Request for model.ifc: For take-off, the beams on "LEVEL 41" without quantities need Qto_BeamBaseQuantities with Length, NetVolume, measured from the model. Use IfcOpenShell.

First a look at what the model holds.

```python
import ifcopenshell
import ifcopenshell.util.element
import ifcopenshell.util.unit

model = ifcopenshell.open("model.ifc")
print(model.schema)
for unit_type in ("LENGTHUNIT", "AREAUNIT", "VOLUMEUNIT"):
    print(unit_type, ifcopenshell.util.unit.calculate_unit_scale(model, unit_type))
storey = next(s for s in model.by_type("IfcBuildingStorey") if s.Name == "LEVEL 41")
beams = [e for e in ifcopenshell.util.element.get_decomposition(storey) if e.is_a("IfcBeam")]
for e in sorted(beams, key=lambda e: e.id()):
    print(e.id(), e.is_a(), e.Name, list(ifcopenshell.util.element.get_psets(e, qtos_only=True)), sep=" | ")
```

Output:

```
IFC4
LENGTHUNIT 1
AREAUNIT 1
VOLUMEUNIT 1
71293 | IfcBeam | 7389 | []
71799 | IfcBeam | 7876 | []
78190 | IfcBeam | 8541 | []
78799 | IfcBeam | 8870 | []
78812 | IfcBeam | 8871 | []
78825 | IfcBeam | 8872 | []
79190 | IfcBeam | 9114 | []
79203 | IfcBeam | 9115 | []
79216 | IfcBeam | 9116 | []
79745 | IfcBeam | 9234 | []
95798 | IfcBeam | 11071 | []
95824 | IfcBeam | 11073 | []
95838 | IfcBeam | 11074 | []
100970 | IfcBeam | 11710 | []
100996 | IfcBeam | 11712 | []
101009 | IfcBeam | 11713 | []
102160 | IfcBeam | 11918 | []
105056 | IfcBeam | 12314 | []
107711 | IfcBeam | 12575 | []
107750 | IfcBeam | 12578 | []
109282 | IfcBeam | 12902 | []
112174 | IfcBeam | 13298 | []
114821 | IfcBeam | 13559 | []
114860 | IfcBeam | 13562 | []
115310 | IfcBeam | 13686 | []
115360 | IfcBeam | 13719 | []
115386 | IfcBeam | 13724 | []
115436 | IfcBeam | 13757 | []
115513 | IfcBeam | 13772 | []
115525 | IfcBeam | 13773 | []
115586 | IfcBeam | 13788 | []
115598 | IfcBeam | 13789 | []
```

```python
import ifcopenshell
import ifcopenshell.api.pset
import ifcopenshell.geom
import ifcopenshell.util.element
import ifcopenshell.util.shape
import ifcopenshell.util.unit

model = ifcopenshell.open("model.ifc")
unit_scale = ifcopenshell.util.unit.calculate_unit_scale(model)
volume_scale = ifcopenshell.util.unit.calculate_unit_scale(model, "VOLUMEUNIT")
settings = ifcopenshell.geom.settings()

storey = next(s for s in model.by_type("IfcBuildingStorey") if s.Name == "LEVEL 41")
beams = [e for e in ifcopenshell.util.element.get_decomposition(storey) if e.is_a("IfcBeam")]

for e in sorted(beams, key=lambda e: e.id()):
    if ifcopenshell.util.element.get_psets(e, qtos_only=True, should_inherit=False):
        continue
    # Geometry comes back in metres, in the element's own axes.
    shape = ifcopenshell.geom.create_shape(settings, e)
    values = {
        "Length": ifcopenshell.util.shape.get_max_xyz(shape.geometry) / unit_scale,
        "NetVolume": ifcopenshell.util.shape.get_volume(shape.geometry) / volume_scale,
    }
    qto = ifcopenshell.api.pset.add_qto(model, product=e, name="Qto_BeamBaseQuantities")
    ifcopenshell.api.pset.edit_qto(model, qto=qto, properties=values)
    print(e.id(), {k: round(v, 3) for k, v in values.items()})

model.write("model-out.ifc")
```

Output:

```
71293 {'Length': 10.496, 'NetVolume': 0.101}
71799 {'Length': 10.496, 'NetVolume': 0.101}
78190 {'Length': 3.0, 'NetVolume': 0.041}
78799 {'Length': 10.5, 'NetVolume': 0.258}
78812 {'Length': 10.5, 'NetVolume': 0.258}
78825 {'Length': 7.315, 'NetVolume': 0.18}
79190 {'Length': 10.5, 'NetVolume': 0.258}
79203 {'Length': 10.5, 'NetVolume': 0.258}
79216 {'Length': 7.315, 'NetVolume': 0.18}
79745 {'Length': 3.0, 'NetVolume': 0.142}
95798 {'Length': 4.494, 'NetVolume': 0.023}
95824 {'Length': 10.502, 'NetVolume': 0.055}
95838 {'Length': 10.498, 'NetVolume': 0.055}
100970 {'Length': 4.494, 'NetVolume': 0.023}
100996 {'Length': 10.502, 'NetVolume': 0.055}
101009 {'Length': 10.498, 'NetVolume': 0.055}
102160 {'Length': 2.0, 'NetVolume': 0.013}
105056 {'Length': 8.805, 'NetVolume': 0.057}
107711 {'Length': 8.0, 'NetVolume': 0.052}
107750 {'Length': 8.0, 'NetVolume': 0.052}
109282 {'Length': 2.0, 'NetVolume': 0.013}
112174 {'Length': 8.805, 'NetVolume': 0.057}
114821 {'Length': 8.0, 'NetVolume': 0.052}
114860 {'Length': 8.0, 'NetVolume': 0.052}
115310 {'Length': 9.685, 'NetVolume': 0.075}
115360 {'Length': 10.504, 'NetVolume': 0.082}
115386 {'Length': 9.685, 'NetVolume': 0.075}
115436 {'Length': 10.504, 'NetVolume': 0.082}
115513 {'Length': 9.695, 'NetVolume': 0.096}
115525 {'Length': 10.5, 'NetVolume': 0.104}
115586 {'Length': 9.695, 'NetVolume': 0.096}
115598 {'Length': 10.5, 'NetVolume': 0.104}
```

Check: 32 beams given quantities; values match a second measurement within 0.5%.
